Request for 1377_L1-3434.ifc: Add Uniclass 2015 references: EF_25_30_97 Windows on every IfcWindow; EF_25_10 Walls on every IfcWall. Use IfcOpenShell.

First a look at what the model holds.

```python
import ifcopenshell

model = ifcopenshell.open("1377_L1-3434.ifc")
print(model.schema)
print("classifications:", [c.Name for c in model.by_type("IfcClassification")])
for ifc_class in ("IfcDoor", "IfcRoof", "IfcStair", "IfcWall", "IfcWindow"):
    print(ifc_class, len(model.by_type(ifc_class)))
```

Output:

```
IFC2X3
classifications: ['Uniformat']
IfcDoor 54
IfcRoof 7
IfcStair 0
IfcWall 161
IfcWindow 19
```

```python
import ifcopenshell
import ifcopenshell.api.classification

model = ifcopenshell.open("1377_L1-3434.ifc")

# IFC2X3 requires Source and Edition and has no link from the project to the system.
system = model.create_entity("IfcClassification", Source="NBS", Edition="2015", Name="Uniclass 2015")

codes = {
    "IfcWindow": ("EF_25_30_97", "Windows"),
    "IfcWall": ("EF_25_10", "Walls"),
}
for ifc_class, (code, name) in codes.items():
    products = model.by_type(ifc_class)
    ifcopenshell.api.classification.add_reference(
        model, products=products, classification=system, identification=code, name=name
    )
    print(code, len(products))

model.write("1377_L1-3434_v2.ifc")
```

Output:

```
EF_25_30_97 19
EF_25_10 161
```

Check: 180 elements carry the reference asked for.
